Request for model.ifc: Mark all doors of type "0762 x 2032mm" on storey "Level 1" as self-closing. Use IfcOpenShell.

First a look at what the model holds.

```python
import ifcopenshell
import ifcopenshell.util.element

model = ifcopenshell.open("model.ifc")
print(model.schema)
storey = next(s for s in model.by_type("IfcBuildingStorey") if s.Name == "Level 1")
doors = [e for e in ifcopenshell.util.element.get_decomposition(storey) if e.is_a("IfcDoor")]
seen = {}
for e in doors:
    element_type = ifcopenshell.util.element.get_type(e)
    key = (element_type.Name if element_type != e and element_type else None, ifcopenshell.util.element.get_pset(e, "Pset_DoorCommon", "SelfClosing"))
    seen[key] = seen.get(key, 0) + 1
for (name, value), count in sorted(seen.items(), key=str):
    print(count, "x", name, "|", value)
```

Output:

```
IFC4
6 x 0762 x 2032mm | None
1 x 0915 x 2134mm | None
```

```python
import ifcopenshell
import ifcopenshell.api.pset
import ifcopenshell.util.element

model = ifcopenshell.open("model.ifc")

storey = next(s for s in model.by_type("IfcBuildingStorey") if s.Name == "Level 1")
doors = [e for e in ifcopenshell.util.element.get_decomposition(storey) if e.is_a("IfcDoor")]

count = 0
for e in doors:
    element_type = ifcopenshell.util.element.get_type(e)
    if element_type in (None, e) or element_type.Name != "0762 x 2032mm":
        continue
    # add_pset returns the element's existing set when there is one.
    pset = ifcopenshell.api.pset.add_pset(model, product=e, name="Pset_DoorCommon")
    ifcopenshell.api.pset.edit_pset(model, pset=pset, properties={"SelfClosing": True})
    count += 1

print(count, "doors updated")

model.write("model_updated.ifc")
```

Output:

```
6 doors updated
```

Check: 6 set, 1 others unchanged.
